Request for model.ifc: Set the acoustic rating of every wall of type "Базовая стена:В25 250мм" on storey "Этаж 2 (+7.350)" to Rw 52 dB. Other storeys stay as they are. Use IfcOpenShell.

First a look at what the model holds.

```python
import ifcopenshell
import ifcopenshell.util.element

model = ifcopenshell.open("model.ifc")
print(model.schema)
storey = next(s for s in model.by_type("IfcBuildingStorey") if s.Name == "Этаж 2 (+7.350)")
walls = [e for e in ifcopenshell.util.element.get_decomposition(storey) if e.is_a("IfcWall")]
seen = {}
for e in walls:
    element_type = ifcopenshell.util.element.get_type(e)
    key = (element_type.Name if element_type != e and element_type else None, ifcopenshell.util.element.get_pset(e, "Pset_WallCommon", "AcousticRating"))
    seen[key] = seen.get(key, 0) + 1
for (name, value), count in sorted(seen.items(), key=str):
    print(count, "x", name, "|", value)
```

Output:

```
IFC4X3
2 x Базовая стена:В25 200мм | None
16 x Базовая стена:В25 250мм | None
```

```python
import ifcopenshell
import ifcopenshell.api.pset
import ifcopenshell.util.element

model = ifcopenshell.open("model.ifc")

storey = next(s for s in model.by_type("IfcBuildingStorey") if s.Name == "Этаж 2 (+7.350)")
walls = [e for e in ifcopenshell.util.element.get_decomposition(storey) if e.is_a("IfcWall")]

count = 0
for e in walls:
    element_type = ifcopenshell.util.element.get_type(e)
    if element_type in (None, e) or element_type.Name != "Базовая стена:В25 250мм":
        continue
    # add_pset returns the element's existing set when there is one.
    pset = ifcopenshell.api.pset.add_pset(model, product=e, name="Pset_WallCommon")
    ifcopenshell.api.pset.edit_pset(model, pset=pset, properties={"AcousticRating": "Rw 52 dB"})
    count += 1

print(count, "walls updated")

model.write("model_updated.ifc")
```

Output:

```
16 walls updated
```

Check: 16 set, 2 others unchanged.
